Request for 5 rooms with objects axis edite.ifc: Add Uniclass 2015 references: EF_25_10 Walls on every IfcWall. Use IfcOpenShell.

First a look at what the model holds.

```python
import ifcopenshell

model = ifcopenshell.open("5 rooms with objects axis edite.ifc")
print(model.schema)
print("classifications:", [c.Name for c in model.by_type("IfcClassification")])
for ifc_class in ("IfcDoor", "IfcRoof", "IfcStair", "IfcWall", "IfcWindow"):
    print(ifc_class, len(model.by_type(ifc_class)))
```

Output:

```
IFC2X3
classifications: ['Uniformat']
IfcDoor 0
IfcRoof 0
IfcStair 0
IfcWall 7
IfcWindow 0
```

```python
import ifcopenshell
import ifcopenshell.api.classification

model = ifcopenshell.open("5 rooms with objects axis edite.ifc")

# IFC2X3 requires Source and Edition and has no link from the project to the system.
system = model.create_entity("IfcClassification", Source="NBS", Edition="2015", Name="Uniclass 2015")

codes = {
    "IfcWall": ("EF_25_10", "Walls"),
}
for ifc_class, (code, name) in codes.items():
    products = model.by_type(ifc_class)
    ifcopenshell.api.classification.add_reference(
        model, products=products, classification=system, identification=code, name=name
    )
    print(code, len(products))

model.write("5 rooms with objects axis edite_edited.ifc")
```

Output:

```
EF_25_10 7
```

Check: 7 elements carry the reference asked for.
